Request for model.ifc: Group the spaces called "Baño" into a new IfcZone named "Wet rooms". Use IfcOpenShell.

First a look at what the model holds.

```python
import ifcopenshell

model = ifcopenshell.open("model.ifc")
print(model.schema)
seen = {}
for space in model.by_type("IfcSpace"):
    seen[space.LongName] = seen.get(space.LongName, 0) + 1
for name, count in sorted(seen.items(), key=str):
    print(count, "x", name)
print("zones:", [z.Name for z in model.by_type("IfcZone")][:20])
```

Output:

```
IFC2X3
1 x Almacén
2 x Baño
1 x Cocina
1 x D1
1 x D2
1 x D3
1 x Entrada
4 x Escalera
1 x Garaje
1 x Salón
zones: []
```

```python
import ifcopenshell
import ifcopenshell.api.group
import ifcopenshell.api.root

model = ifcopenshell.open("model.ifc")

names = {"Baño"}
spaces = [s for s in model.by_type("IfcSpace") if s.LongName in names]

zone = ifcopenshell.api.root.create_entity(model, ifc_class="IfcZone", name="Wet rooms")
ifcopenshell.api.group.assign_group(model, products=spaces, group=zone)
print(len(spaces), "spaces in", zone.Name)

model.write("model_v2.ifc")
```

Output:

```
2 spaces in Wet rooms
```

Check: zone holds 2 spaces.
